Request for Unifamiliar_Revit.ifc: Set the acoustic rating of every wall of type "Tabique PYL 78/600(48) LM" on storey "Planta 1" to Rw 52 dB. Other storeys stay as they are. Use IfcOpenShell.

First a look at what the model holds.

```python
import ifcopenshell
import ifcopenshell.util.element

model = ifcopenshell.open("Unifamiliar_Revit.ifc")
print(model.schema)
storey = next(s for s in model.by_type("IfcBuildingStorey") if s.Name == "Planta 1")
walls = [e for e in ifcopenshell.util.element.get_decomposition(storey) if e.is_a("IfcWall")]
seen = {}
for e in walls:
    element_type = ifcopenshell.util.element.get_type(e)
    key = (element_type.Name if element_type != e and element_type else None, ifcopenshell.util.element.get_pset(e, "Pset_WallCommon", "AcousticRating"))
    seen[key] = seen.get(key, 0) + 1
for (name, value), count in sorted(seen.items(), key=str):
    print(count, "x", name, "|", value)
```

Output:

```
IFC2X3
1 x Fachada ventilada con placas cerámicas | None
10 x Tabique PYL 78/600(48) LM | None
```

```python
import ifcopenshell
import ifcopenshell.api.pset
import ifcopenshell.util.element

model = ifcopenshell.open("Unifamiliar_Revit.ifc")

storey = next(s for s in model.by_type("IfcBuildingStorey") if s.Name == "Planta 1")
walls = [e for e in ifcopenshell.util.element.get_decomposition(storey) if e.is_a("IfcWall")]

count = 0
for e in walls:
    element_type = ifcopenshell.util.element.get_type(e)
    if element_type in (None, e) or element_type.Name != "Tabique PYL 78/600(48) LM":
        continue
    # add_pset returns the element's existing set when there is one.
    pset = ifcopenshell.api.pset.add_pset(model, product=e, name="Pset_WallCommon")
    ifcopenshell.api.pset.edit_pset(model, pset=pset, properties={"AcousticRating": "Rw 52 dB"})
    count += 1

print(count, "walls updated")

model.write("Unifamiliar_Revit_edited.ifc")
```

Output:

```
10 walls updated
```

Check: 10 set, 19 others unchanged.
